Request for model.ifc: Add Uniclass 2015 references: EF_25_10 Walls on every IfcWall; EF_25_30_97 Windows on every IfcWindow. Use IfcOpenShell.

First a look at what the model holds.

```python
import ifcopenshell

model = ifcopenshell.open("model.ifc")
print(model.schema)
print("classifications:", [c.Name for c in model.by_type("IfcClassification")])
for ifc_class in ("IfcDoor", "IfcRoof", "IfcStair", "IfcWall", "IfcWindow"):
    print(ifc_class, len(model.by_type(ifc_class)))
```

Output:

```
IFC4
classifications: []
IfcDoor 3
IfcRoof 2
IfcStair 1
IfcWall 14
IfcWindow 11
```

```python
import ifcopenshell
import ifcopenshell.api.classification

model = ifcopenshell.open("model.ifc")

system = ifcopenshell.api.classification.add_classification(model, classification="Uniclass 2015")

codes = {
    "IfcWall": ("EF_25_10", "Walls"),
    "IfcWindow": ("EF_25_30_97", "Windows"),
}
for ifc_class, (code, name) in codes.items():
    products = model.by_type(ifc_class)
    ifcopenshell.api.classification.add_reference(
        model, products=products, classification=system, identification=code, name=name
    )
    print(code, len(products))

model.write("model_updated.ifc")
```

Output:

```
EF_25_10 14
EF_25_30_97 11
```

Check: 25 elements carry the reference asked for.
